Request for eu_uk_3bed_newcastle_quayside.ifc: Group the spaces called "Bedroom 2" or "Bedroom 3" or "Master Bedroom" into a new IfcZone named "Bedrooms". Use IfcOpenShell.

First a look at what the model holds.

```python
import ifcopenshell

model = ifcopenshell.open("eu_uk_3bed_newcastle_quayside.ifc")
print(model.schema)
seen = {}
for space in model.by_type("IfcSpace"):
    seen[space.LongName] = seen.get(space.LongName, 0) + 1
for name, count in sorted(seen.items(), key=str):
    print(count, "x", name)
print("zones:", [z.Name for z in model.by_type("IfcZone")][:20])
```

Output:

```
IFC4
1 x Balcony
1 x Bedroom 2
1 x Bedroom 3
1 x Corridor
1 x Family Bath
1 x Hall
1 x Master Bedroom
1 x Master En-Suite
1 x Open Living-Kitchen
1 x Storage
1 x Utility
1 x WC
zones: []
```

```python
import ifcopenshell
import ifcopenshell.api.group
import ifcopenshell.api.root

model = ifcopenshell.open("eu_uk_3bed_newcastle_quayside.ifc")

names = {"Bedroom 2", "Bedroom 3", "Master Bedroom"}
spaces = [s for s in model.by_type("IfcSpace") if s.LongName in names]

zone = ifcopenshell.api.root.create_entity(model, ifc_class="IfcZone", name="Bedrooms")
ifcopenshell.api.group.assign_group(model, products=spaces, group=zone)
print(len(spaces), "spaces in", zone.Name)

model.write("eu_uk_3bed_newcastle_quayside-out.ifc")
```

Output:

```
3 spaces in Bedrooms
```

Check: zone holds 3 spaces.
